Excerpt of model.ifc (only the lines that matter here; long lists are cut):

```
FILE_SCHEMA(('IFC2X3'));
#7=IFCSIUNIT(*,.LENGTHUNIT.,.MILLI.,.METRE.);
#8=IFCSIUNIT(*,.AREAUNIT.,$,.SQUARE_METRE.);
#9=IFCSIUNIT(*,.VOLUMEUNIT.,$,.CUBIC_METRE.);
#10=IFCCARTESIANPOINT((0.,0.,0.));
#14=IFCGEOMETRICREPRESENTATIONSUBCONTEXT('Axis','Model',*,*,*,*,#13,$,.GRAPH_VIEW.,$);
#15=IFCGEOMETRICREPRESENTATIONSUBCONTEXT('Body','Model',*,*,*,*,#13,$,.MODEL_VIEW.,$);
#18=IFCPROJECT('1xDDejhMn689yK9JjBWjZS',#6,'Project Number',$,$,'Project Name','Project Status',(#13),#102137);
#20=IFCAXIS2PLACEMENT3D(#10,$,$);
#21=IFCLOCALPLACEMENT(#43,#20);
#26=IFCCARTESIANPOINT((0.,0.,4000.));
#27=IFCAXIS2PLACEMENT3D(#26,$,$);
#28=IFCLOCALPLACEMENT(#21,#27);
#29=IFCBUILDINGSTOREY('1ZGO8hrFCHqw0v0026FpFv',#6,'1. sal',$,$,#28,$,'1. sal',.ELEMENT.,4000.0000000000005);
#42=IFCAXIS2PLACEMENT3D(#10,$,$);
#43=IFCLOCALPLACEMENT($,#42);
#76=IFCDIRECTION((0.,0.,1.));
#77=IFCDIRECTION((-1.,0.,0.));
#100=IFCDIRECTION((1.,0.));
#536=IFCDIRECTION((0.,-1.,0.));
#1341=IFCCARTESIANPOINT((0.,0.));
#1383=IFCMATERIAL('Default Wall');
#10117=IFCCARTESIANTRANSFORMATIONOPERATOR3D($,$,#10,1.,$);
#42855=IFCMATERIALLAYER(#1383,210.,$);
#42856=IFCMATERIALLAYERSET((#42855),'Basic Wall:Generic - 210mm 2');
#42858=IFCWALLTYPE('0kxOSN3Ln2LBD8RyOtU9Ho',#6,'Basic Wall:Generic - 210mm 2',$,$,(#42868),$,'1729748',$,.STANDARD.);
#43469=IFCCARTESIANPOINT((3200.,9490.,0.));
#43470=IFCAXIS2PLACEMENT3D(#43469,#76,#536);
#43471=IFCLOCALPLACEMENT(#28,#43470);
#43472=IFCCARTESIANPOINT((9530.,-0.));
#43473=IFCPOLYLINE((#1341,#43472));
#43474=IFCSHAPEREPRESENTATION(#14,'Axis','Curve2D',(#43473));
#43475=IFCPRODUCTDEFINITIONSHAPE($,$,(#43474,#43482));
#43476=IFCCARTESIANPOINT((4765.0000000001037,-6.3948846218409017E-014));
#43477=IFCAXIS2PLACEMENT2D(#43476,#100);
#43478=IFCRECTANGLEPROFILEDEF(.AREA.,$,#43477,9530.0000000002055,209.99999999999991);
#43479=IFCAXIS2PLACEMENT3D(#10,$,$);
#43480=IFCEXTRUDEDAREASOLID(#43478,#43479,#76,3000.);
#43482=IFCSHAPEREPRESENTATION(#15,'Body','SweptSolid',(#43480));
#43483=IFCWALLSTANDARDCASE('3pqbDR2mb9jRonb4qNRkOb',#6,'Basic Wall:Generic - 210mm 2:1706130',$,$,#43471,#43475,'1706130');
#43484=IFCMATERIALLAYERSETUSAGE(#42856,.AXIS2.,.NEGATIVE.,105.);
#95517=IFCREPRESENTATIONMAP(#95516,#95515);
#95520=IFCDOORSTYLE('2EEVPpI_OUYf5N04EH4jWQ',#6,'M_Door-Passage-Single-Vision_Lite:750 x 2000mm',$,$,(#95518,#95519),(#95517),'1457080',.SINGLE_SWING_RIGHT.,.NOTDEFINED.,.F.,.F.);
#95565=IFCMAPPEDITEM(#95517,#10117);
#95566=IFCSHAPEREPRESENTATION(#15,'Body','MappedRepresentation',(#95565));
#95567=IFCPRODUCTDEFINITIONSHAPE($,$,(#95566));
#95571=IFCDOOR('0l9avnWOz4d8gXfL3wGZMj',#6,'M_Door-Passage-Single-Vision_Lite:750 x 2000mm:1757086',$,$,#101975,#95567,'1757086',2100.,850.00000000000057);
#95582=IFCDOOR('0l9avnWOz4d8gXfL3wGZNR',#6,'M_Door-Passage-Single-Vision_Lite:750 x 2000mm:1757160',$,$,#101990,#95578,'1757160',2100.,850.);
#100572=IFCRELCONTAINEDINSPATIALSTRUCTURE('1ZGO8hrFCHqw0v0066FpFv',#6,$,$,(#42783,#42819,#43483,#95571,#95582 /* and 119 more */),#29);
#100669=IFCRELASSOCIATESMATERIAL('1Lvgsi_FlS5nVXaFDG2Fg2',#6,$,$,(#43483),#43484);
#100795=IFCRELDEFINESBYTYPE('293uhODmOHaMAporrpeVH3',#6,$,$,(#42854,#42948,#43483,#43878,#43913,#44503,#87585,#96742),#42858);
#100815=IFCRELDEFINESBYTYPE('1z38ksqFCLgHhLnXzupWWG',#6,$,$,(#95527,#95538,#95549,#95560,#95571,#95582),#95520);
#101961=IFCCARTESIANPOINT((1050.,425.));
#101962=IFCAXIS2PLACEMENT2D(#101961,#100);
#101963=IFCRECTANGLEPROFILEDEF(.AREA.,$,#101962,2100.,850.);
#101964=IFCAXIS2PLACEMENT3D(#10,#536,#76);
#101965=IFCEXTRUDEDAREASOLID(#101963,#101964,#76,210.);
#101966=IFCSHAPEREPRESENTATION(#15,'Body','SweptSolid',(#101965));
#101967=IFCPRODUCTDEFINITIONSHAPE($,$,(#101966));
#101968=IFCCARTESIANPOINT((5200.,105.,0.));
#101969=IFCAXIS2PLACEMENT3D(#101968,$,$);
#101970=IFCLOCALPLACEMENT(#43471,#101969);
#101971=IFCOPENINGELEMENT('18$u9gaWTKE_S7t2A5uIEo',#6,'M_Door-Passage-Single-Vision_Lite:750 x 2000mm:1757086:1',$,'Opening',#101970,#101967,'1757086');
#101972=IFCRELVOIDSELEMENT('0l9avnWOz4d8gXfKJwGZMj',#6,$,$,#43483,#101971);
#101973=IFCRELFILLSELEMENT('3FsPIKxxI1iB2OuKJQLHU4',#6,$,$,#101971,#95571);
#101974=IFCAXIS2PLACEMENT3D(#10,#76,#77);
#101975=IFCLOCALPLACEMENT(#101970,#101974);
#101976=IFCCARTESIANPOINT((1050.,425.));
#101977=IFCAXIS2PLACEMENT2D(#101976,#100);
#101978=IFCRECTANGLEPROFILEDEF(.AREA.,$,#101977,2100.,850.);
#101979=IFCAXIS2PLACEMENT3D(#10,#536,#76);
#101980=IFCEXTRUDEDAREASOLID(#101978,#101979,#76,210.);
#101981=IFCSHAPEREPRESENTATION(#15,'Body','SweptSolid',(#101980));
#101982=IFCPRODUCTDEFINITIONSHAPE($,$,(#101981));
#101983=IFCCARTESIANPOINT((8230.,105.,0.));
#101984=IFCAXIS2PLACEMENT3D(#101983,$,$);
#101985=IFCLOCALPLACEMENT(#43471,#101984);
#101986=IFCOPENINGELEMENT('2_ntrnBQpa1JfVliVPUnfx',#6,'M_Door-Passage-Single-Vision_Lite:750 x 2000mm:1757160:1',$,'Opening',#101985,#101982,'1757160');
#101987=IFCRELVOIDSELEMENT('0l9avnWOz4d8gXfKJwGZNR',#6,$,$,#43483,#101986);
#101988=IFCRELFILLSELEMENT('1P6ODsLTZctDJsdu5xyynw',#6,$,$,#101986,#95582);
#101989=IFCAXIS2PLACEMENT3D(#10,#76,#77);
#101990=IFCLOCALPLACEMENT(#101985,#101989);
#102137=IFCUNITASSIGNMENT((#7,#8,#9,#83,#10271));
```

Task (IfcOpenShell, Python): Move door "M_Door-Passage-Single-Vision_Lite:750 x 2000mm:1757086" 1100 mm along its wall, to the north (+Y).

```python
import ifcopenshell
import ifcopenshell.api.geometry
import ifcopenshell.util.placement

model = ifcopenshell.open("model.ifc")

door = model.by_id(95571)
opening = door.FillsVoids[0].RelatingOpeningElement
wall = opening.VoidsElements[0].RelatingBuildingElement

wall_matrix = ifcopenshell.util.placement.get_local_placement(wall.ObjectPlacement)
shift = wall_matrix[:3, 0] * -1100.0
before = ifcopenshell.util.placement.get_local_placement(door.ObjectPlacement)[:3, 3].copy()

# The door is placed relative to its opening, so it follows when the opening moves.
matrix = ifcopenshell.util.placement.get_local_placement(opening.ObjectPlacement)
matrix[:3, 3] += shift
ifcopenshell.api.geometry.edit_object_placement(
    model, product=opening, matrix=matrix, is_si=False, should_transform_children=True
)

after = ifcopenshell.util.placement.get_local_placement(door.ObjectPlacement)[:3, 3]
print("door moved by", (after - before).round(3) + 0.0)

model.write("model_v2.ifc")
```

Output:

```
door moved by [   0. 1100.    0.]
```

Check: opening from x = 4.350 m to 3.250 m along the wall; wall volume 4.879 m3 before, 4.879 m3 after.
